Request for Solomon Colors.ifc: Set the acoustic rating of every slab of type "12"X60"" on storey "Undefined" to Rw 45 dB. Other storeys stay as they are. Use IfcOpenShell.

First a look at what the model holds.

```python
import ifcopenshell
import ifcopenshell.util.element

model = ifcopenshell.open("Solomon Colors.ifc")
print(model.schema)
storey = next(s for s in model.by_type("IfcBuildingStorey") if s.Name == "Undefined")
slabs = [e for e in ifcopenshell.util.element.get_decomposition(storey) if e.is_a("IfcSlab")]
seen = {}
for e in slabs:
    element_type = ifcopenshell.util.element.get_type(e)
    key = (element_type.Name if element_type != e and element_type else None, ifcopenshell.util.element.get_pset(e, "Pset_SlabCommon", "AcousticRating"))
    seen[key] = seen.get(key, 0) + 1
for (name, value), count in sorted(seen.items(), key=str):
    print(count, "x", name, "|", value)
```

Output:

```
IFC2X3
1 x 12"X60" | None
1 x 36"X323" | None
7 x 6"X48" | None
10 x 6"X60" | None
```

```python
import ifcopenshell
import ifcopenshell.api.pset
import ifcopenshell.util.element

model = ifcopenshell.open("Solomon Colors.ifc")

storey = next(s for s in model.by_type("IfcBuildingStorey") if s.Name == "Undefined")
slabs = [e for e in ifcopenshell.util.element.get_decomposition(storey) if e.is_a("IfcSlab")]

count = 0
for e in slabs:
    element_type = ifcopenshell.util.element.get_type(e)
    if element_type in (None, e) or element_type.Name != '12"X60"':
        continue
    # add_pset returns the element's existing set when there is one.
    pset = ifcopenshell.api.pset.add_pset(model, product=e, name="Pset_SlabCommon")
    ifcopenshell.api.pset.edit_pset(model, pset=pset, properties={"AcousticRating": "Rw 45 dB"})
    count += 1

print(count, "slabs updated")

model.write("Solomon Colors_edited.ifc")
```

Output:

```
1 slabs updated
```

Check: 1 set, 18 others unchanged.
